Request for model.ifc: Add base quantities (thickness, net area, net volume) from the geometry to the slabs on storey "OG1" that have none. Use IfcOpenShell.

First a look at what the model holds.

```python
import ifcopenshell
import ifcopenshell.util.element
import ifcopenshell.util.unit

model = ifcopenshell.open("model.ifc")
print(model.schema)
for unit_type in ("LENGTHUNIT", "AREAUNIT", "VOLUMEUNIT"):
    print(unit_type, ifcopenshell.util.unit.calculate_unit_scale(model, unit_type))
storey = next(s for s in model.by_type("IfcBuildingStorey") if s.Name == "OG1")
slabs = [e for e in ifcopenshell.util.element.get_decomposition(storey) if e.is_a("IfcSlab")]
for e in sorted(slabs, key=lambda e: e.id()):
    print(e.id(), e.is_a(), e.Name, list(ifcopenshell.util.element.get_psets(e, qtos_only=True)), sep=" | ")
```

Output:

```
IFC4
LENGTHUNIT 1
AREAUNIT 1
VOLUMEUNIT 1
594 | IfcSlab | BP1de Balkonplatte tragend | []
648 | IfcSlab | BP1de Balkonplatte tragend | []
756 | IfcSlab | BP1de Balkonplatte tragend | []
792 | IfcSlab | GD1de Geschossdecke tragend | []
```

```python
import ifcopenshell
import ifcopenshell.api.pset
import ifcopenshell.geom
import ifcopenshell.util.element
import ifcopenshell.util.shape
import ifcopenshell.util.unit

model = ifcopenshell.open("model.ifc")
unit_scale = ifcopenshell.util.unit.calculate_unit_scale(model)
area_scale = ifcopenshell.util.unit.calculate_unit_scale(model, "AREAUNIT")
volume_scale = ifcopenshell.util.unit.calculate_unit_scale(model, "VOLUMEUNIT")
settings = ifcopenshell.geom.settings()

storey = next(s for s in model.by_type("IfcBuildingStorey") if s.Name == "OG1")
slabs = [e for e in ifcopenshell.util.element.get_decomposition(storey) if e.is_a("IfcSlab")]

for e in sorted(slabs, key=lambda e: e.id()):
    if ifcopenshell.util.element.get_psets(e, qtos_only=True, should_inherit=False):
        continue
    # Geometry comes back in metres, in the element's own axes.
    shape = ifcopenshell.geom.create_shape(settings, e)
    values = {
        "Width": ifcopenshell.util.shape.get_z(shape.geometry) / unit_scale,
        "NetArea": ifcopenshell.util.shape.get_footprint_area(shape.geometry) / area_scale,
        "NetVolume": ifcopenshell.util.shape.get_volume(shape.geometry) / volume_scale,
    }
    qto = ifcopenshell.api.pset.add_qto(model, product=e, name="Qto_SlabBaseQuantities")
    ifcopenshell.api.pset.edit_qto(model, qto=qto, properties=values)
    print(e.id(), {k: round(v, 3) for k, v in values.items()})

model.write("model_v2.ifc")
```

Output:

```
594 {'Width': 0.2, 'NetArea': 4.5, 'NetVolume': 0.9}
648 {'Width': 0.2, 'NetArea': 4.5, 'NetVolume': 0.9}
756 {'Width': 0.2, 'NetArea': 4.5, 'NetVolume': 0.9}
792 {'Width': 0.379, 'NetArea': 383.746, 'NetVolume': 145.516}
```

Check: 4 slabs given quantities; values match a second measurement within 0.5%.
